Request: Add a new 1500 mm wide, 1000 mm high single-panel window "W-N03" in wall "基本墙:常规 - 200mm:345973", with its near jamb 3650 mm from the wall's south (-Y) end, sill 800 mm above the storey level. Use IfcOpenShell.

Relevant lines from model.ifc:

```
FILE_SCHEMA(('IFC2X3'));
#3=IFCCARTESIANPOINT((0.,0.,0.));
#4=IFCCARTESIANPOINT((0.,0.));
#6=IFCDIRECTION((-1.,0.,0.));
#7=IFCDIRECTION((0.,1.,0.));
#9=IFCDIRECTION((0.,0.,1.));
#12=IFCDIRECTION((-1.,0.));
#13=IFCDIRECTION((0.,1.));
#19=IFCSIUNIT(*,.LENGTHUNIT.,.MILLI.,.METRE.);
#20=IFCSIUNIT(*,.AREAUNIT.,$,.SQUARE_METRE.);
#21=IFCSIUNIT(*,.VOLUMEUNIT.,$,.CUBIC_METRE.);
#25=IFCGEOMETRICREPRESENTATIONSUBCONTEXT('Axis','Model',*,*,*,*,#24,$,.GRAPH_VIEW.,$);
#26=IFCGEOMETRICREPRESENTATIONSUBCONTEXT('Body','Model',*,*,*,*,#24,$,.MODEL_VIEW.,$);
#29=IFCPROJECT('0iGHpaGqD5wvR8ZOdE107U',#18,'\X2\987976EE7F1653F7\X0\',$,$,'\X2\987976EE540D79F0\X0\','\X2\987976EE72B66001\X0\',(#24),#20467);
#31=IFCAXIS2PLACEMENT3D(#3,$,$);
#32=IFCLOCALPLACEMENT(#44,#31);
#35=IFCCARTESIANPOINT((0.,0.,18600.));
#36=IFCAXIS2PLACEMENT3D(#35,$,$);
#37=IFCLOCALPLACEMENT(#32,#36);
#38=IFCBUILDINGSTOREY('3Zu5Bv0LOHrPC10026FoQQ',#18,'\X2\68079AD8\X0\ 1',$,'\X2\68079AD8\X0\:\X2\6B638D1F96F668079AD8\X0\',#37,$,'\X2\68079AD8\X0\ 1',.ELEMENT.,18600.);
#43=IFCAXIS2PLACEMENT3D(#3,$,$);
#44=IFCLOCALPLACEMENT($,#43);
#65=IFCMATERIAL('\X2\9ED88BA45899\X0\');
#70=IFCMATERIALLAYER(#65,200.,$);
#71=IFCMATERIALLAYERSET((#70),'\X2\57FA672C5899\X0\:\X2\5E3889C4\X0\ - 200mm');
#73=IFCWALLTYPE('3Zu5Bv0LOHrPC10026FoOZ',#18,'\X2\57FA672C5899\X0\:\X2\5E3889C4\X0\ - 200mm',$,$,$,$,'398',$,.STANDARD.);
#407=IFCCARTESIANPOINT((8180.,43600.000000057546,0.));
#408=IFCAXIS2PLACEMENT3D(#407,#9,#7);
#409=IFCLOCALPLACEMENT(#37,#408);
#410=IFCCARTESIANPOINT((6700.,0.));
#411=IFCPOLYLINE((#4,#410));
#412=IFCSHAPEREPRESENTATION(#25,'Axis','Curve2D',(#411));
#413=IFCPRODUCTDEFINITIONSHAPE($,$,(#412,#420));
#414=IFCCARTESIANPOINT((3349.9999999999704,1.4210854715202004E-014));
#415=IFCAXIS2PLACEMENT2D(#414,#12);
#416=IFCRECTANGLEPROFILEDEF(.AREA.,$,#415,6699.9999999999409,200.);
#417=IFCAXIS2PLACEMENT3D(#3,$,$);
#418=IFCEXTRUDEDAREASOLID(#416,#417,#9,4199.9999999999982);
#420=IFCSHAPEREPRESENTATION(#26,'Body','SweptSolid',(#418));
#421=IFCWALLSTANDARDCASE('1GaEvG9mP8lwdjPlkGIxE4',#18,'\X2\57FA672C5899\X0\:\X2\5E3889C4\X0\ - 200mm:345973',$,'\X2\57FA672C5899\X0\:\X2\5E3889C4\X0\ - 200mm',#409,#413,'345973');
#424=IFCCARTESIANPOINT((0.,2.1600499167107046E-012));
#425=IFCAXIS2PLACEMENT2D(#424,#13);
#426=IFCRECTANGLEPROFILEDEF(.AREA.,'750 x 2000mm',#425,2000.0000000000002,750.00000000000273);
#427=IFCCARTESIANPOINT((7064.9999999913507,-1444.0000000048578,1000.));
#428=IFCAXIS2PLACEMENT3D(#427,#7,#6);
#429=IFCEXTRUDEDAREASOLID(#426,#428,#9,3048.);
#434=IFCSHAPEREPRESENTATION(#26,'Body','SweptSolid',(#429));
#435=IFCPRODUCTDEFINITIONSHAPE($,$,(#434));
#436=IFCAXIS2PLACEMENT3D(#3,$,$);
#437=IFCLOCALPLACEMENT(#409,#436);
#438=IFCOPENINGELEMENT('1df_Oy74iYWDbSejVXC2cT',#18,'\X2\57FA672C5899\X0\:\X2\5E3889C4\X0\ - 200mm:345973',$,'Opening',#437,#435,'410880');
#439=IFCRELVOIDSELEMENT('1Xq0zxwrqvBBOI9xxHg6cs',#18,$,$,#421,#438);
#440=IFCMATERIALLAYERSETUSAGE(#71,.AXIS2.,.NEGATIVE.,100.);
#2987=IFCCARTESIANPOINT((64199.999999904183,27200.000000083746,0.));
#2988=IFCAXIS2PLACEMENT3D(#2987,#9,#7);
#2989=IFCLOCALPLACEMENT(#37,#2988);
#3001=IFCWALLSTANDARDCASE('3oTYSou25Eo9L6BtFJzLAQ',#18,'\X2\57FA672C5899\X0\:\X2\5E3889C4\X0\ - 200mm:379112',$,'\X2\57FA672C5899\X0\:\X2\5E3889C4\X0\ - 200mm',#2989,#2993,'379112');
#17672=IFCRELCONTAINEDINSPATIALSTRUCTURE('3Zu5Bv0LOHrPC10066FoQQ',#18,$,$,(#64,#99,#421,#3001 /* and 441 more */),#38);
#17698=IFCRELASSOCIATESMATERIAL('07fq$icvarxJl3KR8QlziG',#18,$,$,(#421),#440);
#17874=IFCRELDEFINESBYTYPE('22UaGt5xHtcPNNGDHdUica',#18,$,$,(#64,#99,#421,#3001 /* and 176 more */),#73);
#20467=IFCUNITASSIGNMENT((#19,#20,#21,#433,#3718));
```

```python
import numpy as np
import ifcopenshell
import ifcopenshell.api.feature
import ifcopenshell.api.geometry
import ifcopenshell.api.root
import ifcopenshell.api.spatial
import ifcopenshell.api.type
import ifcopenshell.geom
import ifcopenshell.util.element
import ifcopenshell.util.placement
import ifcopenshell.util.representation
import ifcopenshell.util.shape
import ifcopenshell.util.unit

model = ifcopenshell.open("model.ifc")
unit_scale = ifcopenshell.util.unit.calculate_unit_scale(model)
settings = ifcopenshell.geom.settings()


def volume(element):
    """Net volume in cubic metres, openings subtracted."""
    shape = ifcopenshell.geom.create_shape(settings, element)
    return ifcopenshell.util.shape.get_volume(shape.geometry)


wall = model.by_id(421)
storey = ifcopenshell.util.element.get_container(wall, ifc_class="IfcBuildingStorey")
context = ifcopenshell.util.representation.get_context(model, "Model", "Body", "MODEL_VIEW")
before = volume(wall)

width, height, from_end, sill = 1.5, 1, 3.65, 0.8  # metres

# The wall runs along its own X axis, and the end named is its -X end.
wall_shape = ifcopenshell.geom.create_shape(settings, wall)
x, y, z = ifcopenshell.util.shape.get_vertices(wall_shape.geometry).T
start = x.min() + from_end
face, thickness = float(y.min()), float(y.max() - y.min())
wall_matrix = ifcopenshell.util.placement.get_local_placement(wall.ObjectPlacement)
level = ifcopenshell.util.placement.get_local_placement(storey.ObjectPlacement)[2, 3]


def in_wall(x, y):
    """Placement at x, y metres in the wall's axes, at sill height."""
    matrix = wall_matrix.copy()
    matrix[:, 3] = wall_matrix @ np.array([x / unit_scale, y / unit_scale, 0.0, 1.0])
    matrix[2, 3] = level + sill / unit_scale
    return matrix


# Opening: a box that overshoots both wall faces by 50 mm.
opening = ifcopenshell.api.root.create_entity(model, ifc_class="IfcOpeningElement")
box = ifcopenshell.api.geometry.add_wall_representation(
    model, context=context, length=width, height=height, thickness=thickness + 0.1
)
ifcopenshell.api.geometry.assign_representation(model, product=opening, representation=box)
ifcopenshell.api.geometry.edit_object_placement(model, product=opening, matrix=in_wall(start, face - 0.05), is_si=False)
ifcopenshell.api.feature.add_feature(model, feature=opening, element=wall)

window = ifcopenshell.api.root.create_entity(model, ifc_class="IfcWindow", name="W-N03")
window.OverallWidth, window.OverallHeight = width / unit_scale, height / unit_scale
body = ifcopenshell.api.geometry.add_window_representation(
    model,
    context=context,
    overall_width=window.OverallWidth,
    overall_height=window.OverallHeight,
    partition_type="SINGLE_PANEL",
)
ifcopenshell.api.geometry.assign_representation(model, product=window, representation=body)
ifcopenshell.api.spatial.assign_container(model, products=[window], relating_structure=storey)
fills = ifcopenshell.api.feature.add_filling(model, opening=opening, element=window)
fills.OwnerHistory = window.OwnerHistory  # required in IFC2X3

# IFC2X3 keeps the operation on the window style.
style = ifcopenshell.api.root.create_entity(model, ifc_class="IfcWindowStyle", name="W-N03")
style.OperationType, style.ConstructionType = "SINGLE_PANEL", "NOTDEFINED"
style.ParameterTakesPrecedence = style.Sizeable = False
ifcopenshell.api.type.assign_type(model, related_objects=[window], relating_type=style)

# Centre the window in the wall's thickness.
ifcopenshell.api.geometry.edit_object_placement(model, product=window, matrix=in_wall(start, face), is_si=False)
window_shape = ifcopenshell.geom.create_shape(settings, window)
depth = ifcopenshell.util.shape.get_vertices(window_shape.geometry)[:, 1]
offset = face + thickness / 2 - (depth.min() + depth.max()) / 2
ifcopenshell.api.geometry.edit_object_placement(model, product=window, matrix=in_wall(start, offset), is_si=False)

after = volume(wall)

print(f"wall volume {before:.3f} -> {after:.3f} m3")

model.write("model_edited.ifc")
```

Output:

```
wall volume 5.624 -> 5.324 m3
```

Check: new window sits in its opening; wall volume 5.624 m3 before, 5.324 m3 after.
